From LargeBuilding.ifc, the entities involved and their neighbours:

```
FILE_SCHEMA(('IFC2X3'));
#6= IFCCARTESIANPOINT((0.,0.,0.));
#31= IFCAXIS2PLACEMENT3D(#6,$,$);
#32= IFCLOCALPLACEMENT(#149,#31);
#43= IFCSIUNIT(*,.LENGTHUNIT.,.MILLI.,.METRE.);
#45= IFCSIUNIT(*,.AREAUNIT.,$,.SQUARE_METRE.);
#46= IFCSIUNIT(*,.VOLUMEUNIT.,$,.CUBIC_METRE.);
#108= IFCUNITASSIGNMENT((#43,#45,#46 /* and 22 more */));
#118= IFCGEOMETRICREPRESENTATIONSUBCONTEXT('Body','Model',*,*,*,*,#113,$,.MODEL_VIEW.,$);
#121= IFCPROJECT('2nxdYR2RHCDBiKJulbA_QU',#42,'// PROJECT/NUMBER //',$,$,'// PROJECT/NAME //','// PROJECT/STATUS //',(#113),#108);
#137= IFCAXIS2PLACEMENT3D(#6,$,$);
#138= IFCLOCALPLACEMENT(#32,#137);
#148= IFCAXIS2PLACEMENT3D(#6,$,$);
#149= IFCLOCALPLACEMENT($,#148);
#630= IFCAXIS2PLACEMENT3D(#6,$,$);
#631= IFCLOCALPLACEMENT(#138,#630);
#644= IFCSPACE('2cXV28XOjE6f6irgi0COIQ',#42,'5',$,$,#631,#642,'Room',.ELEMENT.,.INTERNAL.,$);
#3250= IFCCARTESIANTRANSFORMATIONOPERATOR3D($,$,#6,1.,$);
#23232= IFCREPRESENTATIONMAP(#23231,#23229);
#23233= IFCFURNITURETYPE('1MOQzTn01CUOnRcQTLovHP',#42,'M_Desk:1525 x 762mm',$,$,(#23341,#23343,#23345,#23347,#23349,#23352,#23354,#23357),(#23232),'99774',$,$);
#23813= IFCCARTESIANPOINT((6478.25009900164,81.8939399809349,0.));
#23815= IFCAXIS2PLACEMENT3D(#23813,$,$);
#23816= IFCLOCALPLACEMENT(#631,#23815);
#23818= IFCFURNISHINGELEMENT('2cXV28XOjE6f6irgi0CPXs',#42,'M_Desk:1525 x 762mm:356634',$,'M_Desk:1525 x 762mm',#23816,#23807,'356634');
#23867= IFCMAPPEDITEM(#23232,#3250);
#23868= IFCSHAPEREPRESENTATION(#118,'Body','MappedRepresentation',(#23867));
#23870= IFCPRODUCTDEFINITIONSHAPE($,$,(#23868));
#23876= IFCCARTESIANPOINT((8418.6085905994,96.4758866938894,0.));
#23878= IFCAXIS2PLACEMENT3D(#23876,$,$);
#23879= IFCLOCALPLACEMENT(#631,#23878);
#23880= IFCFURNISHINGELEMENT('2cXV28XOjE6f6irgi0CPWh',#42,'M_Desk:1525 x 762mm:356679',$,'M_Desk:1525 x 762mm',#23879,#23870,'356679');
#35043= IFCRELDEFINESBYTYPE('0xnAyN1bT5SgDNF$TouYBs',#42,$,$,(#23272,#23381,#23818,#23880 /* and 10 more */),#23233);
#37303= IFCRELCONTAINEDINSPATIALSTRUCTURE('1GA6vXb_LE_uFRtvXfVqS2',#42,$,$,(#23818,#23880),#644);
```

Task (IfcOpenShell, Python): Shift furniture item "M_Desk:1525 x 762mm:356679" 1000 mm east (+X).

```python
import ifcopenshell
import ifcopenshell.api.geometry
import ifcopenshell.util.placement

model = ifcopenshell.open("LargeBuilding.ifc")

item = model.by_guid("2cXV28XOjE6f6irgi0CPWh")
matrix = ifcopenshell.util.placement.get_local_placement(item.ObjectPlacement)
matrix[0, 3] += 1000.0
ifcopenshell.api.geometry.edit_object_placement(model, product=item, matrix=matrix, is_si=False)

print(ifcopenshell.util.placement.get_local_placement(item.ObjectPlacement).round(3) + 0.0)

model.write("LargeBuilding-out.ifc")
```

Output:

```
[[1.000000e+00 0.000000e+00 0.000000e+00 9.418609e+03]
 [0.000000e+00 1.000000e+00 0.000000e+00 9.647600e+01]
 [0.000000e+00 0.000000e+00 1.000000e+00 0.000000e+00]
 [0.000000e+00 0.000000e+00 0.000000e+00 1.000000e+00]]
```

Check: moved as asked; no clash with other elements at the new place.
